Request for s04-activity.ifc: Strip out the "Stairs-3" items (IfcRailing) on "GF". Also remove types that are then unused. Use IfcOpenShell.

First a look at what the model holds.

```python
import ifcopenshell
import ifcopenshell.util.element

model = ifcopenshell.open("s04-activity.ifc")
print(model.schema)
storey = next(s for s in model.by_type("IfcBuildingStorey") if s.Name == "GF")
railings = [e for e in ifcopenshell.util.element.get_decomposition(storey) if e.is_a("IfcRailing")]
seen = {}
for e in railings:
    element_type = ifcopenshell.util.element.get_type(e)
    name = element_type.Name if element_type not in (None, e) else None
    seen[name] = seen.get(name, 0) + 1
for name, count in sorted(seen.items(), key=str):
    print(count, "x", name)
```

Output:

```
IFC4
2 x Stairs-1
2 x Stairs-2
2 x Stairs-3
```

```python
import ifcopenshell
import ifcopenshell.api.root
import ifcopenshell.util.element

model = ifcopenshell.open("s04-activity.ifc")

storey = next(s for s in model.by_type("IfcBuildingStorey") if s.Name == "GF")
railings = [e for e in ifcopenshell.util.element.get_decomposition(storey) if e.is_a("IfcRailing")]
targets = [e for e in railings if (t := ifcopenshell.util.element.get_type(e)) not in (None, e) and t.Name == "Stairs-3"]
types = {ifcopenshell.util.element.get_type(e) for e in targets} - {None, *targets}

for e in targets:
    ifcopenshell.api.root.remove_product(model, product=e)
print(len(targets), "removed")

unused = [t for t in types if not ifcopenshell.util.element.get_types(t)]
for t in unused:
    ifcopenshell.api.root.remove_product(model, product=t)
print(len(unused), "unused types removed")

model.write("s04-activity_updated.ifc")
```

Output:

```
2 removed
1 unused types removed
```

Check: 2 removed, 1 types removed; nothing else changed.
